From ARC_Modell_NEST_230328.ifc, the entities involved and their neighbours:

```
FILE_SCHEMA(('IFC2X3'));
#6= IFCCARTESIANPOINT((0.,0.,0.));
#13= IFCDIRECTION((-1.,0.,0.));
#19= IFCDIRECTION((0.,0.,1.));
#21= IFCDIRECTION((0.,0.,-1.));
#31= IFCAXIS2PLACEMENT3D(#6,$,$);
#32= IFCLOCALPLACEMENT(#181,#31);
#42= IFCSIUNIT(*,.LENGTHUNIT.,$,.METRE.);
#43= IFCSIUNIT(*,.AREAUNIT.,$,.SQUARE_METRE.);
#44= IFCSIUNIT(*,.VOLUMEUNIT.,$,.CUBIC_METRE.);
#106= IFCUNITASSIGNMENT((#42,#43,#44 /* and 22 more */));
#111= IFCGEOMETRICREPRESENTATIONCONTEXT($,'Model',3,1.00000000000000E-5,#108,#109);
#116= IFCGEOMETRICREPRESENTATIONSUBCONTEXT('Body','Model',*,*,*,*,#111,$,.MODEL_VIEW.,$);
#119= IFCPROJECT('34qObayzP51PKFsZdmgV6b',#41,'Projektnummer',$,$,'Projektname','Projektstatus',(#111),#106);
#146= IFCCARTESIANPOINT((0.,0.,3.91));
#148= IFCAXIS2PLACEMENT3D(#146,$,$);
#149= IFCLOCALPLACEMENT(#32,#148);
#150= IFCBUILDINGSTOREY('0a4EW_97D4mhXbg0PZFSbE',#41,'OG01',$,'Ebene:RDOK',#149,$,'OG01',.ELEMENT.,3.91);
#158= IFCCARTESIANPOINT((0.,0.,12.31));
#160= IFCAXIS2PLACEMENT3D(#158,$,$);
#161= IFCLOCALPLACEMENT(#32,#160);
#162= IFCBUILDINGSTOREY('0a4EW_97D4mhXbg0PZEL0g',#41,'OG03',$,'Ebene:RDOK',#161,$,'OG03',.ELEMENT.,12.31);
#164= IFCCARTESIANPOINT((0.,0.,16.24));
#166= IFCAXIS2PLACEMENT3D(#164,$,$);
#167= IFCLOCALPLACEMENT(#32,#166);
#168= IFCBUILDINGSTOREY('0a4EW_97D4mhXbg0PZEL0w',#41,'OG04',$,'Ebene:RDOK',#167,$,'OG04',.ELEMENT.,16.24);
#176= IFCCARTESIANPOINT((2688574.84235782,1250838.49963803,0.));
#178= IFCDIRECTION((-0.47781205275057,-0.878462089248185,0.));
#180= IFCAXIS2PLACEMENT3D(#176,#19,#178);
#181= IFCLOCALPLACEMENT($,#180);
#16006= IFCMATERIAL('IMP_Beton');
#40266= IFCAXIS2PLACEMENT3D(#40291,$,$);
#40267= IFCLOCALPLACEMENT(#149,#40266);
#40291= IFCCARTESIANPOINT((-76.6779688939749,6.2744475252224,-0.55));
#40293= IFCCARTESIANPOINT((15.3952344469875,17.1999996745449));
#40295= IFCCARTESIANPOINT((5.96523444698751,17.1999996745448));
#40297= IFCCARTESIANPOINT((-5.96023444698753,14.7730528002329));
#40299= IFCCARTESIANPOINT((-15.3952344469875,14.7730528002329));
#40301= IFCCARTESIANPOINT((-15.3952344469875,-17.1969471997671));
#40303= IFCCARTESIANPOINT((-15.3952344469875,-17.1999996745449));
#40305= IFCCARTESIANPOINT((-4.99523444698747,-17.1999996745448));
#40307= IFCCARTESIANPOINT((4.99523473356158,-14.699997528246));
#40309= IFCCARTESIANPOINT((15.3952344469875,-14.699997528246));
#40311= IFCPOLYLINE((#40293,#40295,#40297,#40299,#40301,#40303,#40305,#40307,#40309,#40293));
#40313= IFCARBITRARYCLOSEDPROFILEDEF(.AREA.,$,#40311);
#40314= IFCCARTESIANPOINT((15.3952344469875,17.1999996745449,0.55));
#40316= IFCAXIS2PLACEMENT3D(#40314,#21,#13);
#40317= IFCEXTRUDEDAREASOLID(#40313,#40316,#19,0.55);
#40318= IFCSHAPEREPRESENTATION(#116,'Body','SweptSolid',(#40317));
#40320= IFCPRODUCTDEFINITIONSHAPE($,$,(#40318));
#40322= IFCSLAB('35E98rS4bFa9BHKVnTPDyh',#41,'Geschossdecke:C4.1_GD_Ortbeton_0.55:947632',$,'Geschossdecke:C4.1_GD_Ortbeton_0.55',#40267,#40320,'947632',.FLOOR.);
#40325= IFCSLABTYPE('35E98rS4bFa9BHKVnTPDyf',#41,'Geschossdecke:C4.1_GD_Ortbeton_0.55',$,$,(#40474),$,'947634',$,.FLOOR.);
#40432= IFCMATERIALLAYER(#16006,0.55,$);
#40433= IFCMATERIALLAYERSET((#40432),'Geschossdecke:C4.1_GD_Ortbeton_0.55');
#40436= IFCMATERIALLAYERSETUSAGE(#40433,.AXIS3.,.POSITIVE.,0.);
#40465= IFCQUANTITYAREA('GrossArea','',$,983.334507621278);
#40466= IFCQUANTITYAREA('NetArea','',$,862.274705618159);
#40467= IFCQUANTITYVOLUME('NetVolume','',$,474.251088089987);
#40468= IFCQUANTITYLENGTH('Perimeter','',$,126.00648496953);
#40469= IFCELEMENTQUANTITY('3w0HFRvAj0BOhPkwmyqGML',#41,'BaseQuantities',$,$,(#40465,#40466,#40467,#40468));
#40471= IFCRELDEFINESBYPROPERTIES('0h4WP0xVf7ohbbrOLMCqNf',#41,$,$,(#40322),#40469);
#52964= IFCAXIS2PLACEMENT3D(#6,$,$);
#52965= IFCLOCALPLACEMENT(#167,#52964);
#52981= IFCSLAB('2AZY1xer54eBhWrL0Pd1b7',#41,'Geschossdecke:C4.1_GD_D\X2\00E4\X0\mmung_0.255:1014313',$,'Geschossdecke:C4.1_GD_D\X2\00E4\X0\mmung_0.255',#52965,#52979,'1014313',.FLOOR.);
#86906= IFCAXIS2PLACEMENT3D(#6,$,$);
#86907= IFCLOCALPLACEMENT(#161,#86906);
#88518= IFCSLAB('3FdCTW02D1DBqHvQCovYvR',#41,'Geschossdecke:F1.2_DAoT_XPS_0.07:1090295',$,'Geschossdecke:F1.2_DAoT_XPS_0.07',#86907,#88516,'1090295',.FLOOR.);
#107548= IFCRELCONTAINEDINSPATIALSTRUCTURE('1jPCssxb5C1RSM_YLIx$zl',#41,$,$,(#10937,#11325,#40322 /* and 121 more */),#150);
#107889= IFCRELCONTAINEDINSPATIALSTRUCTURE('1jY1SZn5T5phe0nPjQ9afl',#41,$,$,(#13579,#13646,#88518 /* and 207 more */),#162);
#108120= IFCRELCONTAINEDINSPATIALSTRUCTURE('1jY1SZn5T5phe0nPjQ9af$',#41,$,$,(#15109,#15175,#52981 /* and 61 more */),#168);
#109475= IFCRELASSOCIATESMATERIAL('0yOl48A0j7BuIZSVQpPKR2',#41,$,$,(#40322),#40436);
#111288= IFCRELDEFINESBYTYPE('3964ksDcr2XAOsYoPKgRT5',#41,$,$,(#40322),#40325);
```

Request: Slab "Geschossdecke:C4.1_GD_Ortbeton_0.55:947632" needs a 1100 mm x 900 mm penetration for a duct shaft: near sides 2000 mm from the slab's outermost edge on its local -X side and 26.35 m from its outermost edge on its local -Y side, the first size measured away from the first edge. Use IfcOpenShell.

```python
import numpy as np
import ifcopenshell
import ifcopenshell.api.feature
import ifcopenshell.api.geometry
import ifcopenshell.api.pset
import ifcopenshell.api.root
import ifcopenshell.geom
import ifcopenshell.util.element
import ifcopenshell.util.placement
import ifcopenshell.util.representation
import ifcopenshell.util.shape
import ifcopenshell.util.unit

model = ifcopenshell.open("ARC_Modell_NEST_230328.ifc")
unit_scale = ifcopenshell.util.unit.calculate_unit_scale(model)
area_scale = ifcopenshell.util.unit.calculate_unit_scale(model, "AREAUNIT")
volume_scale = ifcopenshell.util.unit.calculate_unit_scale(model, "VOLUMEUNIT")
settings = ifcopenshell.geom.settings()


def volume(element):
    """Net volume in cubic metres, openings subtracted."""
    shape = ifcopenshell.geom.create_shape(settings, element)
    return ifcopenshell.util.shape.get_volume(shape.geometry)


slab = model.by_guid("35E98rS4bFa9BHKVnTPDyh")
before = volume(slab)

# Extent in the slab's own axes, in metres. The edges named are its -X and -Y sides.
slab_shape = ifcopenshell.geom.create_shape(settings, slab)
vertices = ifcopenshell.util.shape.get_vertices(slab_shape.geometry)
x_min, y_min, bottom = vertices.min(axis=0)
top = vertices[:, 2].max()

opening = ifcopenshell.api.root.create_entity(model, ifc_class="IfcOpeningElement", name="Duct shaft opening")
context = ifcopenshell.util.representation.get_context(model, "Model", "Body", "MODEL_VIEW")
width, depth = 1.1, 0.9
outline = [(0.0, 0.0), (width, 0.0), (width, depth), (0.0, depth), (0.0, 0.0)]
# Overshoot both faces by 50 mm so the cut is clean.
shape = ifcopenshell.api.geometry.add_slab_representation(
    model, context=context, depth=top - bottom + 0.1, polyline=outline
)
ifcopenshell.api.geometry.assign_representation(model, product=opening, representation=shape)

matrix = ifcopenshell.util.placement.get_local_placement(slab.ObjectPlacement)
matrix[:, 3] = matrix @ np.append(np.array([x_min + 2, y_min + 26.35, bottom - 0.05]) / unit_scale, 1.0)
ifcopenshell.api.geometry.edit_object_placement(model, product=opening, matrix=matrix, is_si=False)
ifcopenshell.api.feature.add_feature(model, feature=opening, element=slab)

after = volume(slab)

# Update the slab's stored quantities.
qto = model.by_id(ifcopenshell.util.element.get_pset(slab, "BaseQuantities", should_inherit=False)["id"])
ifcopenshell.api.pset.edit_qto(model, qto=qto, properties={
    "NetArea": after / (top - bottom) / area_scale,
    "NetVolume": after / volume_scale,
})

print(f"slab volume {before:.3f} -> {after:.3f} m3")

model.write("ARC_Modell_NEST_230328_rev.ifc")
```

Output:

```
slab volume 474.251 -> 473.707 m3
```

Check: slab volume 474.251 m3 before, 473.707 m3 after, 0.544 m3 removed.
